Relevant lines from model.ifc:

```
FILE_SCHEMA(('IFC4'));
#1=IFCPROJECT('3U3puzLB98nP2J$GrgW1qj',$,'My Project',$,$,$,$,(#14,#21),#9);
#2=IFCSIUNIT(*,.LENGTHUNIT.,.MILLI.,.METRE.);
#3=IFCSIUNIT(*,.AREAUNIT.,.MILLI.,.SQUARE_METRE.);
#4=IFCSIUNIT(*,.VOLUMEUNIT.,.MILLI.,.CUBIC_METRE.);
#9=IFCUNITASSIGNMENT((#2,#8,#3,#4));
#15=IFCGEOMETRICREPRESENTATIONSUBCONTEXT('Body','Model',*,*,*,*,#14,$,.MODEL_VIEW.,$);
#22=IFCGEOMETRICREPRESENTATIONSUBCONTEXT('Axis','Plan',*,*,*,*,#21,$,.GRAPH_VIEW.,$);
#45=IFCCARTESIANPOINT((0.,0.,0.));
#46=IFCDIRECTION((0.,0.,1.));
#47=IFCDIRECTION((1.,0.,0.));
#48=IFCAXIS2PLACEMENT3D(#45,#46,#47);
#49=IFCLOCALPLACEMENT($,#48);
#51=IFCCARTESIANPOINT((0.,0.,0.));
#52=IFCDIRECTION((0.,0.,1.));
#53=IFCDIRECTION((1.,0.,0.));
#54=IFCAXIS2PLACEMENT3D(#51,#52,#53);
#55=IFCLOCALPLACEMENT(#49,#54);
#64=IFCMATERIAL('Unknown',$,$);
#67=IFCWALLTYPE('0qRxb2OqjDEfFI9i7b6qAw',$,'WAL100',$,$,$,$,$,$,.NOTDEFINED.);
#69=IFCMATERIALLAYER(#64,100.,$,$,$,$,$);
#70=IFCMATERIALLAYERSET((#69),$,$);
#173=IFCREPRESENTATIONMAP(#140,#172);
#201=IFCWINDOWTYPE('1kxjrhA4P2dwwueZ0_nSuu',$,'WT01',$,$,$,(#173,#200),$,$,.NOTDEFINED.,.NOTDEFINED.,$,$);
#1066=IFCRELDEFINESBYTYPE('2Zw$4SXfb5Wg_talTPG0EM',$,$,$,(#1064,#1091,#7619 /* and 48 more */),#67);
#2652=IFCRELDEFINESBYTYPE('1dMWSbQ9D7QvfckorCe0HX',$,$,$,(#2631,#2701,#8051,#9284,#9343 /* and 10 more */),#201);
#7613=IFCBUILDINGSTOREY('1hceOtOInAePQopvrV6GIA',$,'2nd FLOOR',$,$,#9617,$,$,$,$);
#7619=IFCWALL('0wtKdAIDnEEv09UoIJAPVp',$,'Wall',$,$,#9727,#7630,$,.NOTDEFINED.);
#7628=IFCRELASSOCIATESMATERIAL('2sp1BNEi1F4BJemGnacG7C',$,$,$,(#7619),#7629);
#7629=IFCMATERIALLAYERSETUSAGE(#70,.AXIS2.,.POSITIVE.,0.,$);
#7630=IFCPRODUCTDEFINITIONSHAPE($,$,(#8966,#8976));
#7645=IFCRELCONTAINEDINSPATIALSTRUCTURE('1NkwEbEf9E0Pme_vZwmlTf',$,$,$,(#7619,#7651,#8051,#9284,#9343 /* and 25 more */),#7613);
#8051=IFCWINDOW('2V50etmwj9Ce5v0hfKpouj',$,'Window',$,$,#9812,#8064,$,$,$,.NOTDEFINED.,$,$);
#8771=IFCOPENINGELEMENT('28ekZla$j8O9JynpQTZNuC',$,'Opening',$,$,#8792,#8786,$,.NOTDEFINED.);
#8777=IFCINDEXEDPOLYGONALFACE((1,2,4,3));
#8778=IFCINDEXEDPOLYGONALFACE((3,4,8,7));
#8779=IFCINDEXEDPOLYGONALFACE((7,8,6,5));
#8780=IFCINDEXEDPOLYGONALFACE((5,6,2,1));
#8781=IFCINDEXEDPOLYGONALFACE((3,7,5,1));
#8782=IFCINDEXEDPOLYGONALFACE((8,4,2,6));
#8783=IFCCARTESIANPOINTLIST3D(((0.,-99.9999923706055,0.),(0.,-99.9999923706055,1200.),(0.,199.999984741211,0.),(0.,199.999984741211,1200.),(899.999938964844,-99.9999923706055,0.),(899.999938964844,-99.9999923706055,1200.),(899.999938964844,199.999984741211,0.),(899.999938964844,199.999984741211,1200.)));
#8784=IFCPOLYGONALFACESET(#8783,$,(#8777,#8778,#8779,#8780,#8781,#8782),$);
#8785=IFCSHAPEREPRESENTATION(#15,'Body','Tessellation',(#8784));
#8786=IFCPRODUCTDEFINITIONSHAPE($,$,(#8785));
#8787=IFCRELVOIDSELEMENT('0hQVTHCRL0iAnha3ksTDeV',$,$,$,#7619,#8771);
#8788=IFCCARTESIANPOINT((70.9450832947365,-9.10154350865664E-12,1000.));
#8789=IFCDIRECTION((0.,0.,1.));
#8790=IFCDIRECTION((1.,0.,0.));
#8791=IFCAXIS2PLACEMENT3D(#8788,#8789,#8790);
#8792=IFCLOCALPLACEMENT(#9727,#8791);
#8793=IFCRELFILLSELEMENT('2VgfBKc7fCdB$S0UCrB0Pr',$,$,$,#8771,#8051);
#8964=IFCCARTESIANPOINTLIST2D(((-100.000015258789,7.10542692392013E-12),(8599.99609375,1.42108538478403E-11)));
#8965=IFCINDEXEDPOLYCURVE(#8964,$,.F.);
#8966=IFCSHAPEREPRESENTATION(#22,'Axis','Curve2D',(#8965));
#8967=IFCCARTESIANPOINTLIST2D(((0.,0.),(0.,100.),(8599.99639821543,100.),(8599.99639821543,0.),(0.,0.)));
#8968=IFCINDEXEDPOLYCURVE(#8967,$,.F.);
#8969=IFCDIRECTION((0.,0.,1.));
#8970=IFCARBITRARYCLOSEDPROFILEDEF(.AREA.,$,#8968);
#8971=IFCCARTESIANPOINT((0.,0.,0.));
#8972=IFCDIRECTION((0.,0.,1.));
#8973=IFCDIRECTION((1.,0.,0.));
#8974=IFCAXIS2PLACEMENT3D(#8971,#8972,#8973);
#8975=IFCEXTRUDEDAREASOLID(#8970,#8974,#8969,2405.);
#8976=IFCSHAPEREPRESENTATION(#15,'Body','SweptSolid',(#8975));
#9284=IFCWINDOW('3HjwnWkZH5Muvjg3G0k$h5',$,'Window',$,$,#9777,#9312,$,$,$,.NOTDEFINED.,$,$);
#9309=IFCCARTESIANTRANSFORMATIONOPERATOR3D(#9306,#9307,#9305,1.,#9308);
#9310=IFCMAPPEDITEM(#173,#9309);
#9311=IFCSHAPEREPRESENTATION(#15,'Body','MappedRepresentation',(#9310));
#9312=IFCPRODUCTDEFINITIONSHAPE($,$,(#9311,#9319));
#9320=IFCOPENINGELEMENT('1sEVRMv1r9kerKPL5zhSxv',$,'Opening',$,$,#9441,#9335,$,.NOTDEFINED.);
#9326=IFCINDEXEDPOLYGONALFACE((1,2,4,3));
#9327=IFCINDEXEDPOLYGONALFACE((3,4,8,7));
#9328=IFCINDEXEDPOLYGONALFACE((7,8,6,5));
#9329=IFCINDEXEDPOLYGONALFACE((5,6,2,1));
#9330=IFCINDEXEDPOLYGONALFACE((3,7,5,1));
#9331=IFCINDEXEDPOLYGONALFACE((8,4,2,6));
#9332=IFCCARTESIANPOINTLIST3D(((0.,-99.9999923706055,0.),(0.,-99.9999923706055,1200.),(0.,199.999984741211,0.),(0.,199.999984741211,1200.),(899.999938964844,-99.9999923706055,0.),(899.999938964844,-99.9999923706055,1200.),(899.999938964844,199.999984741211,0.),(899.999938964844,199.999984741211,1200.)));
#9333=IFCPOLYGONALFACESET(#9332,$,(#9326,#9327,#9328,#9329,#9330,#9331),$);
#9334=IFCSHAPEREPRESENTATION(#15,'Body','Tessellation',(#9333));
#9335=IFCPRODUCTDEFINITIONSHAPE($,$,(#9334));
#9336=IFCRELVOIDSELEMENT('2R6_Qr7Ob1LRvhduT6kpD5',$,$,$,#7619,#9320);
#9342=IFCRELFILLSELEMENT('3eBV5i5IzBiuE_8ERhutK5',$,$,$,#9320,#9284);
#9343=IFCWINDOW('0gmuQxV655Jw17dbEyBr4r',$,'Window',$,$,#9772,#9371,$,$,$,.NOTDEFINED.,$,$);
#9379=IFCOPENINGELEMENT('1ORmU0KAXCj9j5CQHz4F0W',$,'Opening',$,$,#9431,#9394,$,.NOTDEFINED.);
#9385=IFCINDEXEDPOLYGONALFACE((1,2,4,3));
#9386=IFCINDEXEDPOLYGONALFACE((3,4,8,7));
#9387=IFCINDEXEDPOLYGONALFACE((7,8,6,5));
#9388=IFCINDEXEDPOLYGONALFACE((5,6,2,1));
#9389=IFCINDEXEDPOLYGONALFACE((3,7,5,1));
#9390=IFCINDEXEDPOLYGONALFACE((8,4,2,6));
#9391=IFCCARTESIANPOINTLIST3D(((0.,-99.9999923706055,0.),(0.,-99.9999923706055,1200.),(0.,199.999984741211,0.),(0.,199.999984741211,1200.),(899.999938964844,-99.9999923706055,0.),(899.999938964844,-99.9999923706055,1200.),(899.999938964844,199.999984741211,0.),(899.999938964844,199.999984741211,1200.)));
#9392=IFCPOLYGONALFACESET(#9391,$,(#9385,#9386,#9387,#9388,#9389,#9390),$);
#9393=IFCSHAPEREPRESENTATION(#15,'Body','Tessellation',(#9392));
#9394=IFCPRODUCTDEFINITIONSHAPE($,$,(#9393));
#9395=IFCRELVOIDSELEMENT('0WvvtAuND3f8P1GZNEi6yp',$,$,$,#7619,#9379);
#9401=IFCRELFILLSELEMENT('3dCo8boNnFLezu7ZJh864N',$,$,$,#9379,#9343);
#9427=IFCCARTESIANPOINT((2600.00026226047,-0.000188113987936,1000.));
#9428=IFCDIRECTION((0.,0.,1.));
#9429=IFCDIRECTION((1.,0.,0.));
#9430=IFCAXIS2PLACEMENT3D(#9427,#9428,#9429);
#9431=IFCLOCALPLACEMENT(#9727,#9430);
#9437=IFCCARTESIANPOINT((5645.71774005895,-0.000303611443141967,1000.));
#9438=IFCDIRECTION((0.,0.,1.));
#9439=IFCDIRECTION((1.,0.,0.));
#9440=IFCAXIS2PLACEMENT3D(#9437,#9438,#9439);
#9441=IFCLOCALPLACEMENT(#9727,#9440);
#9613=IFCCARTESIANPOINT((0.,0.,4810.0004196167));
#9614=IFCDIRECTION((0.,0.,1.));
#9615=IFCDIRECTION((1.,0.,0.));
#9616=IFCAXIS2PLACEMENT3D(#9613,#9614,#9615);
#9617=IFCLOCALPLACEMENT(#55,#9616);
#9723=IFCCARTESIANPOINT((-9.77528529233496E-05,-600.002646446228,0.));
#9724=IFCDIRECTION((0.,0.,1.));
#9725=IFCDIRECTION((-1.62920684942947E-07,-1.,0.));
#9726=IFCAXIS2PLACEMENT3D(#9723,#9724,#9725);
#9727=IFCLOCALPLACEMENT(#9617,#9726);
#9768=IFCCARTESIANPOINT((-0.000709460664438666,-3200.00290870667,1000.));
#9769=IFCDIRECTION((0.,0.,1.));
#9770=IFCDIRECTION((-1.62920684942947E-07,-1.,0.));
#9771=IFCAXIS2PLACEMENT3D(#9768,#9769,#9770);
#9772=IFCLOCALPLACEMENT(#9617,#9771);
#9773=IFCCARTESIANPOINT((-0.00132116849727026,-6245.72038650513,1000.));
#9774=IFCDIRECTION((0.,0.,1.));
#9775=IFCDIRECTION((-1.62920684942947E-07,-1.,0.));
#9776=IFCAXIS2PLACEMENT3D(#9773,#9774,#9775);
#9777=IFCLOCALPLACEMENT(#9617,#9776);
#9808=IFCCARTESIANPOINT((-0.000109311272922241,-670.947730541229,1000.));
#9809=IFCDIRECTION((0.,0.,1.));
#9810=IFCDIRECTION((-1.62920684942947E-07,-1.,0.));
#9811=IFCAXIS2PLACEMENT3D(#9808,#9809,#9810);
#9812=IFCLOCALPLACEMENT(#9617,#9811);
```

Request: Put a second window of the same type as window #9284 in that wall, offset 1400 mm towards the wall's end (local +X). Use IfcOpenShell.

```python
import ifcopenshell
import ifcopenshell.api.feature
import ifcopenshell.api.geometry
import ifcopenshell.api.root
import ifcopenshell.geom
import ifcopenshell.util.element
import ifcopenshell.util.placement
import ifcopenshell.util.shape

model = ifcopenshell.open("model.ifc")
settings = ifcopenshell.geom.settings()


def volume(element):
    """Net volume in cubic metres, openings subtracted."""
    shape = ifcopenshell.geom.create_shape(settings, element)
    return ifcopenshell.util.shape.get_volume(shape.geometry)


window = model.by_guid("3HjwnWkZH5Muvjg3G0k$h5")
opening = window.FillsVoids[0].RelatingOpeningElement
wall = opening.VoidsElements[0].RelatingBuildingElement
before = volume(wall)
shift = ifcopenshell.util.placement.get_local_placement(wall.ObjectPlacement)[:3, 0] * 1400.0

# copy_class copies the void relationship, type, container and properties, but no geometry.
new_opening = ifcopenshell.api.root.copy_class(model, product=opening)
new_opening.Representation = ifcopenshell.util.element.copy_deep(
    model, opening.Representation, exclude=["IfcGeometricRepresentationContext", "IfcRepresentationMap"]
)
new_window = ifcopenshell.api.root.copy_class(model, product=window)
new_window.Representation = ifcopenshell.util.element.copy_deep(
    model, window.Representation, exclude=["IfcGeometricRepresentationContext", "IfcRepresentationMap"]
)
ifcopenshell.api.feature.add_filling(model, opening=new_opening, element=new_window)

for old, new in ((opening, new_opening), (window, new_window)):
    matrix = ifcopenshell.util.placement.get_local_placement(old.ObjectPlacement)
    matrix[:3, 3] += shift
    ifcopenshell.api.geometry.edit_object_placement(model, product=new, matrix=matrix, is_si=False)

after = volume(wall)

print(f"wall volume {before:.3f} -> {after:.3f} m3")

model.write("model_v2.ifc")
```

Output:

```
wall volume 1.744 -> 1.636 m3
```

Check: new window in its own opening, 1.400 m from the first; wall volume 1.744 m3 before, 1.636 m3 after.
